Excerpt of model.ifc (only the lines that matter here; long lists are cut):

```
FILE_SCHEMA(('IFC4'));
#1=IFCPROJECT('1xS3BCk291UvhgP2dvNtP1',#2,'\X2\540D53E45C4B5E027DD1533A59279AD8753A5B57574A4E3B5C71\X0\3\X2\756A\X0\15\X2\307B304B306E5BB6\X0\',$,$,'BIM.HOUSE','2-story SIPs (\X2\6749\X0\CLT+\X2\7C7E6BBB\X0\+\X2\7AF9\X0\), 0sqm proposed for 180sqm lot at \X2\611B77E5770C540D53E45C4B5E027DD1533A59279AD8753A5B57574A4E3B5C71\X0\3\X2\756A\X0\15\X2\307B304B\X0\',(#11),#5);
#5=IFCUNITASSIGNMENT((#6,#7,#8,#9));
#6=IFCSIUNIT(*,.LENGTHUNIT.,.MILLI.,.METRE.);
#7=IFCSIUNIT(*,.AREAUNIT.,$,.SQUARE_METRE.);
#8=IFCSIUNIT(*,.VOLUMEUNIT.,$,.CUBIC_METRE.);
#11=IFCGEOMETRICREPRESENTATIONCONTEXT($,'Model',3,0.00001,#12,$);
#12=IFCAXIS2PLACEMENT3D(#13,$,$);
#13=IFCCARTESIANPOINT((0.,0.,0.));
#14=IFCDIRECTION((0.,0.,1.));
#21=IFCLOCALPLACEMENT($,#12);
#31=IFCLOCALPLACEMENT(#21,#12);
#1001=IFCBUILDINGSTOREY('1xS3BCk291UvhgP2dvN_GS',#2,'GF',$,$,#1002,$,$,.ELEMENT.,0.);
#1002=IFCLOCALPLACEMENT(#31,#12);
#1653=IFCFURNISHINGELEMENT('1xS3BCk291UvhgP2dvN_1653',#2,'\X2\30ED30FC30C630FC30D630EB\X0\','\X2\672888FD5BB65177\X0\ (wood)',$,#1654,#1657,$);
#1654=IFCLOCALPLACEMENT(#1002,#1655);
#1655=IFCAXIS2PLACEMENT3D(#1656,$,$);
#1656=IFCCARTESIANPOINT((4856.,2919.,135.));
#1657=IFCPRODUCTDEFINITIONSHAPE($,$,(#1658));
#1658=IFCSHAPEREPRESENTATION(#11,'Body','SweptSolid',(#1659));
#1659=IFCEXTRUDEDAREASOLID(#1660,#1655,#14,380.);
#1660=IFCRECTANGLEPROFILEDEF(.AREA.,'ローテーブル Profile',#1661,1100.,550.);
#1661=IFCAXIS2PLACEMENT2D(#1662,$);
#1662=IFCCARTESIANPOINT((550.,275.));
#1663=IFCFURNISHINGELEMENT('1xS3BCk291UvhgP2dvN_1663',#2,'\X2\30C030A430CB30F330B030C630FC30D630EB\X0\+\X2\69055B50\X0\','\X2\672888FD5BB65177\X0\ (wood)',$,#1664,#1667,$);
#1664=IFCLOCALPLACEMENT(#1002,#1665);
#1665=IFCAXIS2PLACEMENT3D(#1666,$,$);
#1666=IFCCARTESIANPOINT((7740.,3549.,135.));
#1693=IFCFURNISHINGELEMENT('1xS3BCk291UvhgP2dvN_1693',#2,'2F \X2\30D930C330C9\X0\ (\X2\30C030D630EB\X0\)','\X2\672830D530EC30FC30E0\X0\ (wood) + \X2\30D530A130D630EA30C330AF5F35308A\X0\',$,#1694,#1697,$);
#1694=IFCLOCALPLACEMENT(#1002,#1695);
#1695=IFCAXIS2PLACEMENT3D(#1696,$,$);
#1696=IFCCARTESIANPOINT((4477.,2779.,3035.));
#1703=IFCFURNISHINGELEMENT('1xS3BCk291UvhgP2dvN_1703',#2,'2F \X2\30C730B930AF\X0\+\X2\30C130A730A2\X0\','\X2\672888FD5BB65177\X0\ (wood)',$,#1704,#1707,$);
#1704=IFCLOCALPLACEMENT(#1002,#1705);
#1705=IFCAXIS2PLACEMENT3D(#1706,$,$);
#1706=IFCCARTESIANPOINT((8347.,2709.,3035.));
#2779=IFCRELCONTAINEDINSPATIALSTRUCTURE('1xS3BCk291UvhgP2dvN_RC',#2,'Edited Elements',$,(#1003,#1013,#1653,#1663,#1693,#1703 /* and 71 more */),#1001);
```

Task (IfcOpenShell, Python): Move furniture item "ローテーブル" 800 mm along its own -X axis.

```python
import ifcopenshell
import ifcopenshell.api.geometry
import ifcopenshell.util.placement
import ifcopenshell.util.unit

model = ifcopenshell.open("model.ifc")
unit_scale = ifcopenshell.util.unit.calculate_unit_scale(model)

item = model.by_guid("1xS3BCk291UvhgP2dvN_1653")
matrix = ifcopenshell.util.placement.get_local_placement(item.ObjectPlacement)
matrix[:3, 3] -= matrix[:3, 0] * 0.8 / unit_scale
ifcopenshell.api.geometry.edit_object_placement(model, product=item, matrix=matrix, is_si=False)

print(ifcopenshell.util.placement.get_local_placement(item.ObjectPlacement).round(3) + 0.0)

model.write("model_updated.ifc")
```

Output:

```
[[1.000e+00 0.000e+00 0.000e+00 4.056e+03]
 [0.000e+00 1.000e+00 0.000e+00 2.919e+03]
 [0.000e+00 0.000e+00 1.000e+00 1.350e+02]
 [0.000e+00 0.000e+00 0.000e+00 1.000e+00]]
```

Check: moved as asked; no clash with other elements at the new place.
